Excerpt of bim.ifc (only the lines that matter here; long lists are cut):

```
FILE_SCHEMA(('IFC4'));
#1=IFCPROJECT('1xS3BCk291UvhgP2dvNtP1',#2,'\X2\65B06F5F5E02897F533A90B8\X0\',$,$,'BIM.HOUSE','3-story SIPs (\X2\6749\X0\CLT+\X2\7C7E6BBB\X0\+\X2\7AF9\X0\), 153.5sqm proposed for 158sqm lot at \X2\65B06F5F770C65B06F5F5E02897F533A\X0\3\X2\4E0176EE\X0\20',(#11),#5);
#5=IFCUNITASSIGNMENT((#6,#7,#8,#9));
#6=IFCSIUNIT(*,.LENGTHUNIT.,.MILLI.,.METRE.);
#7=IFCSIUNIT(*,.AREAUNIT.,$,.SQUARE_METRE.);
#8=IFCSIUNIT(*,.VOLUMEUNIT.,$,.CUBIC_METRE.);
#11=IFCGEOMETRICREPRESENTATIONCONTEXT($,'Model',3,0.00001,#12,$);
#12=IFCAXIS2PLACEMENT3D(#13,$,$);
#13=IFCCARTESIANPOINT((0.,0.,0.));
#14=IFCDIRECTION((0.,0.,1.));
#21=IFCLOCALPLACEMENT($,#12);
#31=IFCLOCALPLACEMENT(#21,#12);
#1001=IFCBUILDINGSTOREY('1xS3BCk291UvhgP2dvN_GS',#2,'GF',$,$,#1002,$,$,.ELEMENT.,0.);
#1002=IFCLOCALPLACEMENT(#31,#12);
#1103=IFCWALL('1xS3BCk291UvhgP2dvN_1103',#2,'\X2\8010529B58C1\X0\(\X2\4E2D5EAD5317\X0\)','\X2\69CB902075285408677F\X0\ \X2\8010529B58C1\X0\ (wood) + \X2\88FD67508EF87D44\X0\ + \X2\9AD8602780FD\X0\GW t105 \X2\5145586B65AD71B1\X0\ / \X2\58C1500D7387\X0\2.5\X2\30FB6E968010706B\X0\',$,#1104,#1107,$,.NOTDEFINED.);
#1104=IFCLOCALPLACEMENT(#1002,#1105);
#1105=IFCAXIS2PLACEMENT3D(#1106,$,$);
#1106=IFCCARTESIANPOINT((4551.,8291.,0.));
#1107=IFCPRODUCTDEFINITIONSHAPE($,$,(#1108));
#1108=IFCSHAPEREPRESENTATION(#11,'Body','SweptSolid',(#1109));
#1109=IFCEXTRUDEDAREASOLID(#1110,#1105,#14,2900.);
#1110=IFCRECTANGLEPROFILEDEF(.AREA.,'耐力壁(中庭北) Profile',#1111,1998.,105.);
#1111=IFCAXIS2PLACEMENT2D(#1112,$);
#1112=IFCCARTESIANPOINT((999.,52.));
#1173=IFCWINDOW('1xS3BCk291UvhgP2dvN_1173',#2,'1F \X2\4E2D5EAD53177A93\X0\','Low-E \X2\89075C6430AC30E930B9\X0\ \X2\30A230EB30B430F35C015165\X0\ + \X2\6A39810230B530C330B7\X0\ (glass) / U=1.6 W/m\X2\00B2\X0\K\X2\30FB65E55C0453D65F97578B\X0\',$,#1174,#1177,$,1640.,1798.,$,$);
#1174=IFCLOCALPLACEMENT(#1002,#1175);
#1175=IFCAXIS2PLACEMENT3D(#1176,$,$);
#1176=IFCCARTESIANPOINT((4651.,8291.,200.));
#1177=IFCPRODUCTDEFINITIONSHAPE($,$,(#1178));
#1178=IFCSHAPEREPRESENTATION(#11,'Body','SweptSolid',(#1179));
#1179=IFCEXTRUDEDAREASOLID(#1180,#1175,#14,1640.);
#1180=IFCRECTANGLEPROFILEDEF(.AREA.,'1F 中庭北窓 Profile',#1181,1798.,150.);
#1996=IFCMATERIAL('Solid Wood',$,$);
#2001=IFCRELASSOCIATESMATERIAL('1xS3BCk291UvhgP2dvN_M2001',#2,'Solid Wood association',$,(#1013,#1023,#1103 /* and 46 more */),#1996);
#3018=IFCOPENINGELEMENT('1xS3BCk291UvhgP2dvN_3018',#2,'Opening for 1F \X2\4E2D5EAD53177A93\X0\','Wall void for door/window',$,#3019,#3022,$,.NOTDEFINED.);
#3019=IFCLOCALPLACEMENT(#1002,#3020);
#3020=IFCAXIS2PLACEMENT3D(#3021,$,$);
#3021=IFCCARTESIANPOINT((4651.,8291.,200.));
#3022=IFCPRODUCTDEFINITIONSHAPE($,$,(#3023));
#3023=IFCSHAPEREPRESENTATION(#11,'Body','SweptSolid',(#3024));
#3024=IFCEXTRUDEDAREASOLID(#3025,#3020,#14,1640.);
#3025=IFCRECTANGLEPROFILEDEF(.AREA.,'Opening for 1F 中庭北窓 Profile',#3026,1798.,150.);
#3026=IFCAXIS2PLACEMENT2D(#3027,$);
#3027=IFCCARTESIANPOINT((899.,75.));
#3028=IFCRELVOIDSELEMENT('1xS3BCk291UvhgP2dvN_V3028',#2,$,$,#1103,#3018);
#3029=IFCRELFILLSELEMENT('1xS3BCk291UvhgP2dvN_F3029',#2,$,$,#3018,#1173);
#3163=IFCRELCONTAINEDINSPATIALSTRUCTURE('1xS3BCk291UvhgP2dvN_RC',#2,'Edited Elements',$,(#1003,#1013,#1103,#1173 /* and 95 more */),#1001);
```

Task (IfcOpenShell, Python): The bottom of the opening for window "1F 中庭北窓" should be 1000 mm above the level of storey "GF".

```python
import numpy as np
import ifcopenshell
import ifcopenshell.api.geometry
import ifcopenshell.geom
import ifcopenshell.util.element
import ifcopenshell.util.placement
import ifcopenshell.util.shape
import ifcopenshell.util.unit

model = ifcopenshell.open("bim.ifc")
unit_scale = ifcopenshell.util.unit.calculate_unit_scale(model)

window = model.by_id(1173)
opening = window.FillsVoids[0].RelatingOpeningElement
storey = ifcopenshell.util.element.get_container(window, ifc_class="IfcBuildingStorey")
level = ifcopenshell.util.placement.get_local_placement(storey.ObjectPlacement)[2, 3]

# The opening's origin need not be at the sill, so measure its lowest point.
shape = ifcopenshell.geom.create_shape(ifcopenshell.geom.settings(), opening)
bottom = ifcopenshell.util.shape.get_shape_bottom_elevation(shape, shape.geometry) / unit_scale
dz = level + 1000.0 - bottom

shift = np.array([0.0, 0.0, dz])
# The window is not placed relative to its opening, so move both.
for product in (opening, window):
    matrix = ifcopenshell.util.placement.get_local_placement(product.ObjectPlacement)
    matrix[:3, 3] += shift
    ifcopenshell.api.geometry.edit_object_placement(model, product=product, matrix=matrix, is_si=False)

print(f"moved by {dz * unit_scale:+.3f} m")

model.write("bim_edited.ifc")
```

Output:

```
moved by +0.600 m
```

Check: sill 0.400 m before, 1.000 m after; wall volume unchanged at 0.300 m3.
